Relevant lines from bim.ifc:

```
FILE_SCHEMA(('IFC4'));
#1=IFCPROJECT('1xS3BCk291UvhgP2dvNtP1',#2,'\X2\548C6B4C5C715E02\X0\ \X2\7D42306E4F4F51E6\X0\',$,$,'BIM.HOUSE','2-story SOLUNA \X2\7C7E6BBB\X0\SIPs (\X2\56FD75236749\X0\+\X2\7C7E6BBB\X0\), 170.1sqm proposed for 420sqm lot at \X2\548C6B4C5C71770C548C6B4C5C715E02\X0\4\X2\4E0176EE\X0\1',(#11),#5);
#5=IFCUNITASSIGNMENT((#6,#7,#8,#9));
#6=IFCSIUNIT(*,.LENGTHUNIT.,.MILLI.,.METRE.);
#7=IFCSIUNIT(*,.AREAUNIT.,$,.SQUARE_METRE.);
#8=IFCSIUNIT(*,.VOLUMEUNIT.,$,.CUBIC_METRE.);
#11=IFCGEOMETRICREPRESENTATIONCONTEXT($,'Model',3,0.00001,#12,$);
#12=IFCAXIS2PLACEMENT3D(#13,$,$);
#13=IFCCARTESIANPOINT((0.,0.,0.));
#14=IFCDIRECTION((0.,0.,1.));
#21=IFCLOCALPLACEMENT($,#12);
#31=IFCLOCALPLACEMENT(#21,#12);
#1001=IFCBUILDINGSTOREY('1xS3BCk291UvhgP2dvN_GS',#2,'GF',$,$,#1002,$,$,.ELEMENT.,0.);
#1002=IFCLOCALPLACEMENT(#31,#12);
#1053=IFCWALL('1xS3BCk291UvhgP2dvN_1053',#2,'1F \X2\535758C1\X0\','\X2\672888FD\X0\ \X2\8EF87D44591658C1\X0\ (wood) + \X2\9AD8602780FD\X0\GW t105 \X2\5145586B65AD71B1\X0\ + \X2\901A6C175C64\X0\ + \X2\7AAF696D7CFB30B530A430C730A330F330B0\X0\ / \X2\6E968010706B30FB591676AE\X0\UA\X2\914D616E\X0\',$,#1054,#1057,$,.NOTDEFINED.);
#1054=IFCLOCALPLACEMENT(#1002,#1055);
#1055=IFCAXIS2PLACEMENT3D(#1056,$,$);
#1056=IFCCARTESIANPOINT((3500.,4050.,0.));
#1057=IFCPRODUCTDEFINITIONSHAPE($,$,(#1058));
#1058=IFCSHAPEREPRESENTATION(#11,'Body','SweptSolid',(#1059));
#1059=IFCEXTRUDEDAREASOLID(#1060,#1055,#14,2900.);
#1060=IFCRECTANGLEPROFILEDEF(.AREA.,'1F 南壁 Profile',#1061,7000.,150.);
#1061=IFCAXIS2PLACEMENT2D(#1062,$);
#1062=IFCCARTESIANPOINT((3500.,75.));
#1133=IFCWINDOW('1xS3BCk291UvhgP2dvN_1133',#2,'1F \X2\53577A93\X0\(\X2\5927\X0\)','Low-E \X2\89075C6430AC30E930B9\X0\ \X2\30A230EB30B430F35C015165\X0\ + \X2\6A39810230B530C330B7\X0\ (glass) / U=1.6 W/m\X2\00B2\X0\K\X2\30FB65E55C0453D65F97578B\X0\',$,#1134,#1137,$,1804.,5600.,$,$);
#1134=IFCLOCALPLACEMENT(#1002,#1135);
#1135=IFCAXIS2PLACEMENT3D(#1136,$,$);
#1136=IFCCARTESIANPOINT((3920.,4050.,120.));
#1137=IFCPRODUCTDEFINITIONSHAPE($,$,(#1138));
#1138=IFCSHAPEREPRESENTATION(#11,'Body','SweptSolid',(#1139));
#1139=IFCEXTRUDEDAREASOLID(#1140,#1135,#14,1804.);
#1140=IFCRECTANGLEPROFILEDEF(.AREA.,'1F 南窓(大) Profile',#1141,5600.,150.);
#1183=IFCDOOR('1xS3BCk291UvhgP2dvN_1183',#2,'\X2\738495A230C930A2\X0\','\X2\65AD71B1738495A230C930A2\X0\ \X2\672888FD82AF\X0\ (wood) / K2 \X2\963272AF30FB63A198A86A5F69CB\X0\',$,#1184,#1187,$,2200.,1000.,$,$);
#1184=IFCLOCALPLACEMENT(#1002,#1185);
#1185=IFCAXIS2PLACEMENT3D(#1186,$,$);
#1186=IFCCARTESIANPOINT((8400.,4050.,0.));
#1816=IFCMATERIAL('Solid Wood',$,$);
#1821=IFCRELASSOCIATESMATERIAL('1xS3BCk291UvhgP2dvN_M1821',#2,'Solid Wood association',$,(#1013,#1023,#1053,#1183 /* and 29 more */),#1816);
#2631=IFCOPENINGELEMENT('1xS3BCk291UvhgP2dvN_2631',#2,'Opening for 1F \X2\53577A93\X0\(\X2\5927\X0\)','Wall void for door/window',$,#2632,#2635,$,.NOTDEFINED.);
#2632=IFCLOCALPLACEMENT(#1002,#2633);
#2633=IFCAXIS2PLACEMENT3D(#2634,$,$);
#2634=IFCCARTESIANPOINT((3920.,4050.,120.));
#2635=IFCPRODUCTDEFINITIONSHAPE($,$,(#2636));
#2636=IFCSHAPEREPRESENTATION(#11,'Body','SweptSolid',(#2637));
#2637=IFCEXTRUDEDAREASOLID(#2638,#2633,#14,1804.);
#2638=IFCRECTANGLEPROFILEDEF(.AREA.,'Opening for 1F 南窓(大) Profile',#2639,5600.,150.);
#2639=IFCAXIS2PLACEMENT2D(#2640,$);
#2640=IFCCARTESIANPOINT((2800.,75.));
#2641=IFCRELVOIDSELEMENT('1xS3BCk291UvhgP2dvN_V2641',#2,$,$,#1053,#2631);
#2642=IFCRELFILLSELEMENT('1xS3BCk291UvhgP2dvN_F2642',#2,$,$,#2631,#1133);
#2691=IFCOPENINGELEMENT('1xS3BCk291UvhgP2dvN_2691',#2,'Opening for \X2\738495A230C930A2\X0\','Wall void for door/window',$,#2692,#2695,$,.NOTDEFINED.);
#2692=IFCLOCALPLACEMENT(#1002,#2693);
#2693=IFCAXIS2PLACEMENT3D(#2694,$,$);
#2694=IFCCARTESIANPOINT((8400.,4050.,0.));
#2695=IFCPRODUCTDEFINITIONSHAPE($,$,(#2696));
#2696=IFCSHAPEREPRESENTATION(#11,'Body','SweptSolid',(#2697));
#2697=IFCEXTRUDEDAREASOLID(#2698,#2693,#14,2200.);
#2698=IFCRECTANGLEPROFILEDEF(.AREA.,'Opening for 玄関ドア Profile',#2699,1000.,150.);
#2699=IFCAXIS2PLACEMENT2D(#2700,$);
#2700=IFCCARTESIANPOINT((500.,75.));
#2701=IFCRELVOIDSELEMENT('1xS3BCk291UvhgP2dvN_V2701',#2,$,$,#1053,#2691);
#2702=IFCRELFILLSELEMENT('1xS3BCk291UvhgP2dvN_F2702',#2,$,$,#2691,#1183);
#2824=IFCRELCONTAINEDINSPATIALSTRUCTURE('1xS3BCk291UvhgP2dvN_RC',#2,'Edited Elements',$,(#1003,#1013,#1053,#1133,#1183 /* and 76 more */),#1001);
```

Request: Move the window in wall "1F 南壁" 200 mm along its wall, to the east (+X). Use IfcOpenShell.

```python
import ifcopenshell
import ifcopenshell.api.geometry
import ifcopenshell.util.placement
import ifcopenshell.util.unit

model = ifcopenshell.open("bim.ifc")
unit_scale = ifcopenshell.util.unit.calculate_unit_scale(model)

window = model.by_id(1133)
opening = window.FillsVoids[0].RelatingOpeningElement
wall = opening.VoidsElements[0].RelatingBuildingElement

wall_matrix = ifcopenshell.util.placement.get_local_placement(wall.ObjectPlacement)
shift = wall_matrix[:3, 0] * 0.2 / unit_scale
before = ifcopenshell.util.placement.get_local_placement(window.ObjectPlacement)[:3, 3].copy()

# The window is not placed relative to its opening, so move both.
for product in (opening, window):
    matrix = ifcopenshell.util.placement.get_local_placement(product.ObjectPlacement)
    matrix[:3, 3] += shift
    ifcopenshell.api.geometry.edit_object_placement(model, product=product, matrix=matrix, is_si=False)

after = ifcopenshell.util.placement.get_local_placement(window.ObjectPlacement)[:3, 3]
print("window moved by", (after - before).round(3) + 0.0)

model.write("bim_rev.ifc")
```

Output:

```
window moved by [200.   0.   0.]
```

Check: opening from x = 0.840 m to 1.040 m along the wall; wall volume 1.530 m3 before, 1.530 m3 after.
